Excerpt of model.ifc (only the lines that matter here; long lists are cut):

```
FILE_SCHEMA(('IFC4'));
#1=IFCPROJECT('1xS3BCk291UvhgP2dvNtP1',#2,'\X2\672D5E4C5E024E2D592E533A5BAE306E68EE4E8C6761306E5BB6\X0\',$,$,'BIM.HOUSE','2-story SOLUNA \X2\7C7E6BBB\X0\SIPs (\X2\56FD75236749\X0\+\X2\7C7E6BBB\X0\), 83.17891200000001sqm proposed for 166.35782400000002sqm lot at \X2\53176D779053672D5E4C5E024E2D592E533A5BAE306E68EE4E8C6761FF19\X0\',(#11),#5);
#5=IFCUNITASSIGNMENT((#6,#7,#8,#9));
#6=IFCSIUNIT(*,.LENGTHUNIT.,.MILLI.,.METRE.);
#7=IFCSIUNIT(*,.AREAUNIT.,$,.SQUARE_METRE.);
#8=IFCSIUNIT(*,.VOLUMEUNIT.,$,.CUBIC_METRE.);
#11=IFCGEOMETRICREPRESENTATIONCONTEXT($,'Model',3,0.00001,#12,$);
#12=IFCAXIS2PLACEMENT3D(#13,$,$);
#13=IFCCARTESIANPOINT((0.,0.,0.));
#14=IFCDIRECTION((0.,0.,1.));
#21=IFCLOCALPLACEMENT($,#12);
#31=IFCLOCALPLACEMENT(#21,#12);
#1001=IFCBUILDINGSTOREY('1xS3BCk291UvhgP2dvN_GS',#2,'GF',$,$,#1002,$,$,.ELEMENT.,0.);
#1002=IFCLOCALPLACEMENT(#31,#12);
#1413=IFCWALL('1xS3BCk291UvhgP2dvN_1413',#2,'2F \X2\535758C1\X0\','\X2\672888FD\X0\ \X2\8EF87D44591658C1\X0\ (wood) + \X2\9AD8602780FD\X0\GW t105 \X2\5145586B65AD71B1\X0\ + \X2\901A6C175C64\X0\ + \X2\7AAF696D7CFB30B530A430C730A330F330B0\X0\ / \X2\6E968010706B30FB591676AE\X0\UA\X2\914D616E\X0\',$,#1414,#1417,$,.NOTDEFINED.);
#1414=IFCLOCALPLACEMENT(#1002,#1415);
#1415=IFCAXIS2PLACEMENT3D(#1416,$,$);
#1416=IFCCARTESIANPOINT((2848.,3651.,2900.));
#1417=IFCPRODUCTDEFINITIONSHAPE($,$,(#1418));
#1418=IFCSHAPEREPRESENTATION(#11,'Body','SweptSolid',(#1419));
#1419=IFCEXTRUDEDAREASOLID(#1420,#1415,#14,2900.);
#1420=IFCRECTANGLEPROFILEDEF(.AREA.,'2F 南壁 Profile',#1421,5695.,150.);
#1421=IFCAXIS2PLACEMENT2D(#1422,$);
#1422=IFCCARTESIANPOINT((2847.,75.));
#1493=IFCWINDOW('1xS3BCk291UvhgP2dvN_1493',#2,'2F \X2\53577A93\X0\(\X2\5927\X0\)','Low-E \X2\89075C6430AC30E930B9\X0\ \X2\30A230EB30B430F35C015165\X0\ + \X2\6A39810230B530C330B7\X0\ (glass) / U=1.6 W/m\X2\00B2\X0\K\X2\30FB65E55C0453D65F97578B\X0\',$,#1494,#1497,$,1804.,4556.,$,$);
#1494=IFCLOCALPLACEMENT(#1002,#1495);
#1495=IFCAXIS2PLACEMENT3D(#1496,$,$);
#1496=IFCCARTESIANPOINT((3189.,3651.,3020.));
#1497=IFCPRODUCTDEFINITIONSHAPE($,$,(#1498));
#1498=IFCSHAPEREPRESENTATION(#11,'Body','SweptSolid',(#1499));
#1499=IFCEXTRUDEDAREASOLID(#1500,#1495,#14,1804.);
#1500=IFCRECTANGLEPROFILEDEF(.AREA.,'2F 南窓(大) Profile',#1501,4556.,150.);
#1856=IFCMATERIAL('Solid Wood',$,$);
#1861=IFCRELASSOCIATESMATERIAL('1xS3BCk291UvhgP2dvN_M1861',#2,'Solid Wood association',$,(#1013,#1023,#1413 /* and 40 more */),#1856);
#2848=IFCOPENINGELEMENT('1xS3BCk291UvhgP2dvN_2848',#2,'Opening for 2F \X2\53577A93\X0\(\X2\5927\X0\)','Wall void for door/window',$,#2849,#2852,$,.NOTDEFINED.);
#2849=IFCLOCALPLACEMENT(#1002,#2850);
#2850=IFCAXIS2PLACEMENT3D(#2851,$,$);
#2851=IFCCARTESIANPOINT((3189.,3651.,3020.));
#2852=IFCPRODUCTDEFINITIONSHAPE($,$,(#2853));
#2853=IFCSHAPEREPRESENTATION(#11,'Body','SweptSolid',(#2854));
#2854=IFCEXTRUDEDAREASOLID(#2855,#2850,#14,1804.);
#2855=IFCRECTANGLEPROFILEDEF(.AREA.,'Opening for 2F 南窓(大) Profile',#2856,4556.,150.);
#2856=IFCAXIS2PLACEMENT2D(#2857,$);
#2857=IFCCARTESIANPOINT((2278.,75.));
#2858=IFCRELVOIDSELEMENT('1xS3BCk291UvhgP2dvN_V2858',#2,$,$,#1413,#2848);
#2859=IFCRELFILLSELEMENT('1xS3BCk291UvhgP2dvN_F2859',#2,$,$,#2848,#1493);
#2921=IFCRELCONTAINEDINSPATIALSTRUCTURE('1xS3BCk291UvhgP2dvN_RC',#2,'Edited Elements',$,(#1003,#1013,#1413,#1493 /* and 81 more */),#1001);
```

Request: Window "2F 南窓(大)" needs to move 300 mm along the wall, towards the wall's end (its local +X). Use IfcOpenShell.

```python
import ifcopenshell
import ifcopenshell.api.geometry
import ifcopenshell.util.placement
import ifcopenshell.util.unit

model = ifcopenshell.open("model.ifc")
unit_scale = ifcopenshell.util.unit.calculate_unit_scale(model)

window = model.by_id(1493)
opening = window.FillsVoids[0].RelatingOpeningElement
wall = opening.VoidsElements[0].RelatingBuildingElement

wall_matrix = ifcopenshell.util.placement.get_local_placement(wall.ObjectPlacement)
shift = wall_matrix[:3, 0] * 0.3 / unit_scale
before = ifcopenshell.util.placement.get_local_placement(window.ObjectPlacement)[:3, 3].copy()

# The window is not placed relative to its opening, so move both.
for product in (opening, window):
    matrix = ifcopenshell.util.placement.get_local_placement(product.ObjectPlacement)
    matrix[:3, 3] += shift
    ifcopenshell.api.geometry.edit_object_placement(model, product=product, matrix=matrix, is_si=False)

after = ifcopenshell.util.placement.get_local_placement(window.ObjectPlacement)[:3, 3]
print("window moved by", (after - before).round(3) + 0.0)

model.write("model_updated.ifc")
```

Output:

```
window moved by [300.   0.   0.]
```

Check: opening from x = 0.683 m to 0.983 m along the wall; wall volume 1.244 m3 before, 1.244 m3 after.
